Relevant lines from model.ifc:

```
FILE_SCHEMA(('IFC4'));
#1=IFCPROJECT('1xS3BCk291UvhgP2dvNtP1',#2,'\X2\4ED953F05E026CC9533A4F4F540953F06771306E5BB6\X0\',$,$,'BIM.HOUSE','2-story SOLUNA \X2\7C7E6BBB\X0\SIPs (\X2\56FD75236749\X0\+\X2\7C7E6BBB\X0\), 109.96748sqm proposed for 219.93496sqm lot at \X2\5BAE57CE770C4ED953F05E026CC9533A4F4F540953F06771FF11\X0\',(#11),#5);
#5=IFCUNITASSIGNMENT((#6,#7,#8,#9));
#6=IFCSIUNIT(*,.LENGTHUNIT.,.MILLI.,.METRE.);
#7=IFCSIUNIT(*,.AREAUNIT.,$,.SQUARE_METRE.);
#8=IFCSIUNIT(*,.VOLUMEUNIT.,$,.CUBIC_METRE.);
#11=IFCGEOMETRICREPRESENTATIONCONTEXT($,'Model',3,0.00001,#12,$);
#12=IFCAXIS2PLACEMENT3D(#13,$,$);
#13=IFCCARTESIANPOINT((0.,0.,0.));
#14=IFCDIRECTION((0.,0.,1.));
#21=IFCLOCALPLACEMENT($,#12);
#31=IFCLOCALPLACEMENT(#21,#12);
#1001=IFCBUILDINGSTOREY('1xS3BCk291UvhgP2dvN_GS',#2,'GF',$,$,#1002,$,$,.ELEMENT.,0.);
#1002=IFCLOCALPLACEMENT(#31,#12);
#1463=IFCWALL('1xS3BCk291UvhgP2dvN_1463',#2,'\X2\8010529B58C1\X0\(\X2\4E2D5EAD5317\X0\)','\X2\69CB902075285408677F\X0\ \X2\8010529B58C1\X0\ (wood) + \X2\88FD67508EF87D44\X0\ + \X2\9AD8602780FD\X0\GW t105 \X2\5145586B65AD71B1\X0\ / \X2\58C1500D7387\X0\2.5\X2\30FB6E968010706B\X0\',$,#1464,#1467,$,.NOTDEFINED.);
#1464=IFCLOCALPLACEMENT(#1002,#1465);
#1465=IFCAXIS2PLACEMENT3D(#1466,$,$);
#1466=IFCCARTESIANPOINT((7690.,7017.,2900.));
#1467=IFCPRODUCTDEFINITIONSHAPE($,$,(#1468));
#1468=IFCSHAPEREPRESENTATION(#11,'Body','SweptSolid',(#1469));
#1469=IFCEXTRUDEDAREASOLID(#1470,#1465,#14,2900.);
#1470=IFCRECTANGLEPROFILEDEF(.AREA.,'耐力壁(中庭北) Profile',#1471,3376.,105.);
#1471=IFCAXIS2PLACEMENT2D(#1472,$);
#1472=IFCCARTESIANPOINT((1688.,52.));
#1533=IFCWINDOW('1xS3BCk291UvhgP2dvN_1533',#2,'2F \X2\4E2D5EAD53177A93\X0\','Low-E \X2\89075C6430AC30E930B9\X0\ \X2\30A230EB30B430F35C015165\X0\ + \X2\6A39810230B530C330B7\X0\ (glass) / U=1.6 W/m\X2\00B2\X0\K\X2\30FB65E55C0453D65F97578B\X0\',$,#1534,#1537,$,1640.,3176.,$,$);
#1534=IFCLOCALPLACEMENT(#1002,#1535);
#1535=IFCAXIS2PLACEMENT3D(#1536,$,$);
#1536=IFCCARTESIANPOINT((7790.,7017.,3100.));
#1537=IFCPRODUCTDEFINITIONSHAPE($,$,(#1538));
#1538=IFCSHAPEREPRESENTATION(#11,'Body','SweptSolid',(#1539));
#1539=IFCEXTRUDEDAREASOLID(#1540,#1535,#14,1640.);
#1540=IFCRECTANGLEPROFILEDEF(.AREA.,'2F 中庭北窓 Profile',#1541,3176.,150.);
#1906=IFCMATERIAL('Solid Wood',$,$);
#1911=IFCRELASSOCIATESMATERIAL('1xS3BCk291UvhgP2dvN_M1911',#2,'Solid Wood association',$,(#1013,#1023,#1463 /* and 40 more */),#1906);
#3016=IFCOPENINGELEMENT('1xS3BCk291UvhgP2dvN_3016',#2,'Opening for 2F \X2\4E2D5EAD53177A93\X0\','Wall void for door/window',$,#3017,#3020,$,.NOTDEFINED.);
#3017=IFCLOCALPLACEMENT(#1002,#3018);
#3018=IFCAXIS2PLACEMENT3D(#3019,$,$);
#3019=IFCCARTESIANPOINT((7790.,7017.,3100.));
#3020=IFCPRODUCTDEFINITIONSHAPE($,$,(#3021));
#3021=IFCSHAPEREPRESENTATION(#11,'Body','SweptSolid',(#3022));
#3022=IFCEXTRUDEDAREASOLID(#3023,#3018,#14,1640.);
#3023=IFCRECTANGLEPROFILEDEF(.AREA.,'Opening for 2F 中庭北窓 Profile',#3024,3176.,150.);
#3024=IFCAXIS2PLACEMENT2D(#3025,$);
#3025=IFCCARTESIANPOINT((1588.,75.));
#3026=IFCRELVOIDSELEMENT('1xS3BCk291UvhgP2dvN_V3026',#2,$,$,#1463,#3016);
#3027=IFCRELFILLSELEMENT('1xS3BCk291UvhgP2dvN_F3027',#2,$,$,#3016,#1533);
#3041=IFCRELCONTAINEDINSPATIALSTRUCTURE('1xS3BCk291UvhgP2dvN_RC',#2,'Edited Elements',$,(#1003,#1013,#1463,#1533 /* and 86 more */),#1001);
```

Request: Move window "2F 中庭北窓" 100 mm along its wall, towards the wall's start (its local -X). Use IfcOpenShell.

```python
import ifcopenshell
import ifcopenshell.api.geometry
import ifcopenshell.util.placement

model = ifcopenshell.open("model.ifc")

window = model.by_guid("1xS3BCk291UvhgP2dvN_1533")
opening = window.FillsVoids[0].RelatingOpeningElement
wall = opening.VoidsElements[0].RelatingBuildingElement

wall_matrix = ifcopenshell.util.placement.get_local_placement(wall.ObjectPlacement)
shift = wall_matrix[:3, 0] * -100.0
before = ifcopenshell.util.placement.get_local_placement(window.ObjectPlacement)[:3, 3].copy()

# The window is not placed relative to its opening, so move both.
for product in (opening, window):
    matrix = ifcopenshell.util.placement.get_local_placement(product.ObjectPlacement)
    matrix[:3, 3] += shift
    ifcopenshell.api.geometry.edit_object_placement(model, product=product, matrix=matrix, is_si=False)

after = ifcopenshell.util.placement.get_local_placement(window.ObjectPlacement)[:3, 3]
print("window moved by", (after - before).round(3) + 0.0)

model.write("model_updated.ifc")
```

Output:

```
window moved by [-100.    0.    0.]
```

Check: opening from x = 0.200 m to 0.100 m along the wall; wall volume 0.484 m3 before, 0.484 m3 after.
